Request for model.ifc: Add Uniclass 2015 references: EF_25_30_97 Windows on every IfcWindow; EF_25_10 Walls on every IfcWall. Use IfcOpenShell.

First a look at what the model holds.

```python
import ifcopenshell

model = ifcopenshell.open("model.ifc")
print(model.schema)
print("classifications:", [c.Name for c in model.by_type("IfcClassification")])
for ifc_class in ("IfcDoor", "IfcRoof", "IfcStair", "IfcWall", "IfcWindow"):
    print(ifc_class, len(model.by_type(ifc_class)))
```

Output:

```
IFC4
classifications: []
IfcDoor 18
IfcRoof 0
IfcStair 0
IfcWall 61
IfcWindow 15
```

```python
import ifcopenshell
import ifcopenshell.api.classification

model = ifcopenshell.open("model.ifc")

system = ifcopenshell.api.classification.add_classification(model, classification="Uniclass 2015")

codes = {
    "IfcWindow": ("EF_25_30_97", "Windows"),
    "IfcWall": ("EF_25_10", "Walls"),
}
for ifc_class, (code, name) in codes.items():
    products = model.by_type(ifc_class)
    ifcopenshell.api.classification.add_reference(
        model, products=products, classification=system, identification=code, name=name
    )
    print(code, len(products))

model.write("model_updated.ifc")
```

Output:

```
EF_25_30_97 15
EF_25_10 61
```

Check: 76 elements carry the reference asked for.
